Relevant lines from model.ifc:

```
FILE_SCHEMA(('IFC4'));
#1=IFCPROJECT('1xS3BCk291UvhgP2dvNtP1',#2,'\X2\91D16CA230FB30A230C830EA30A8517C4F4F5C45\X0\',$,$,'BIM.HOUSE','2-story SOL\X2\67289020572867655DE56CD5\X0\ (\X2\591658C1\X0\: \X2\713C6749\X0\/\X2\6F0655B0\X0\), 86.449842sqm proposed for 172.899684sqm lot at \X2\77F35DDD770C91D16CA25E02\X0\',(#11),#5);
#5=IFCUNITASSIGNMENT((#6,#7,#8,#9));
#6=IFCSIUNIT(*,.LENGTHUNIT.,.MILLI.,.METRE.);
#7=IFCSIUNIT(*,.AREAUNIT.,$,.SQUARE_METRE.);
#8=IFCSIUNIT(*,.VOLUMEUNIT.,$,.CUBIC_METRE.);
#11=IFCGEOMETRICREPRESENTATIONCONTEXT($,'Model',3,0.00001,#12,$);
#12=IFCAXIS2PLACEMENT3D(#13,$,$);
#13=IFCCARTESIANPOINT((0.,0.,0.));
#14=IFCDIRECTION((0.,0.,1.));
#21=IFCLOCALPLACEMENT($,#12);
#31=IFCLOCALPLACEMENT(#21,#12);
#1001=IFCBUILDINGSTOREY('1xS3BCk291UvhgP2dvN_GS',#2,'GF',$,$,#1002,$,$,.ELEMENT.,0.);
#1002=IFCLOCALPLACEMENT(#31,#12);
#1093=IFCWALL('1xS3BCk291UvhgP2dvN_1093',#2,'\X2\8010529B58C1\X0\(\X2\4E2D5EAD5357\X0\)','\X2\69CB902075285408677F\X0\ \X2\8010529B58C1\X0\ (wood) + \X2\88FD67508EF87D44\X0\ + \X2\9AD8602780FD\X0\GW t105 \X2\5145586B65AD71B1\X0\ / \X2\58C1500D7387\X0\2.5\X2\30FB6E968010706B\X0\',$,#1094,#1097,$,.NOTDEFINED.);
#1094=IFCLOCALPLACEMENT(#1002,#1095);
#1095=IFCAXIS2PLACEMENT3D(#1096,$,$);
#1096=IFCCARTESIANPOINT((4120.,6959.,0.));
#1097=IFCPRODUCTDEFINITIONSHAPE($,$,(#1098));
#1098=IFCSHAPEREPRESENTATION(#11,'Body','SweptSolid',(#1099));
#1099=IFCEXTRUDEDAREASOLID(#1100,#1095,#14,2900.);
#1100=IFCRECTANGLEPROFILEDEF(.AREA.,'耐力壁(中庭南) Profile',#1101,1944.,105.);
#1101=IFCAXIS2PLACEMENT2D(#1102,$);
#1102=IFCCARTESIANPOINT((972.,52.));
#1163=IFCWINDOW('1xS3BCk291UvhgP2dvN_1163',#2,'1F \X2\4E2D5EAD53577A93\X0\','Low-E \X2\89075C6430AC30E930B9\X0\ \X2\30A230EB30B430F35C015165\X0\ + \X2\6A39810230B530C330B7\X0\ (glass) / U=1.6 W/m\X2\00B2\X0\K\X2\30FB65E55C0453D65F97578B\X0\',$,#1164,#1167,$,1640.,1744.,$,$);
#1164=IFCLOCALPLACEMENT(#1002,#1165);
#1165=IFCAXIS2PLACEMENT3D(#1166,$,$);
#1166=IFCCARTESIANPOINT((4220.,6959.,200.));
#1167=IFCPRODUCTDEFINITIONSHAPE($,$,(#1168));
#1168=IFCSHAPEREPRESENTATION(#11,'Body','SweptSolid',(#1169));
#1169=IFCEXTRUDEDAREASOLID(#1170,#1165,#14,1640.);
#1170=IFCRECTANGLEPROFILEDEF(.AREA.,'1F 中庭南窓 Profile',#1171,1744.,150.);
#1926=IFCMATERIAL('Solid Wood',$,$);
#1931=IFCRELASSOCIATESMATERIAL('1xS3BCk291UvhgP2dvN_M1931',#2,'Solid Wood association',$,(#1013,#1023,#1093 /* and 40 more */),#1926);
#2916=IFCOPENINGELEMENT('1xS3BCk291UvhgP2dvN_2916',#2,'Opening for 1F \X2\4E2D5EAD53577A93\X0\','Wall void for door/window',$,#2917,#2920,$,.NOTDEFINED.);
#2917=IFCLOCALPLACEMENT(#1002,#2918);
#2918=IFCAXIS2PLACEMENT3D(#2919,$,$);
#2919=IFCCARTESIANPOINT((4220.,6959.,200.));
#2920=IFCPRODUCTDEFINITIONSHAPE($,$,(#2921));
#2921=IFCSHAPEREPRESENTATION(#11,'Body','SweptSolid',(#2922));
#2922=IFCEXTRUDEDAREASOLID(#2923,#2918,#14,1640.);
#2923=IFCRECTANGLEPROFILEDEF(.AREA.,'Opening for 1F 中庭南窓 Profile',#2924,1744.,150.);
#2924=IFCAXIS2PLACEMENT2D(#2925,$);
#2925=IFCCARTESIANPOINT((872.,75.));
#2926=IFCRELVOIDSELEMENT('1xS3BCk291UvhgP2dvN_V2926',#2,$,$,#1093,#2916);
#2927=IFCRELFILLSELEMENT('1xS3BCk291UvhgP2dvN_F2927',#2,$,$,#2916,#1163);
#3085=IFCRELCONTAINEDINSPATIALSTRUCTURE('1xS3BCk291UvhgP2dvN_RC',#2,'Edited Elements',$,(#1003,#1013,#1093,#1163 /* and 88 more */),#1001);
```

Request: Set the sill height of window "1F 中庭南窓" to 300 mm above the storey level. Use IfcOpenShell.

```python
import numpy as np
import ifcopenshell
import ifcopenshell.api.geometry
import ifcopenshell.geom
import ifcopenshell.util.element
import ifcopenshell.util.placement
import ifcopenshell.util.shape
import ifcopenshell.util.unit

model = ifcopenshell.open("model.ifc")
unit_scale = ifcopenshell.util.unit.calculate_unit_scale(model)

window = model.by_guid("1xS3BCk291UvhgP2dvN_1163")
opening = window.FillsVoids[0].RelatingOpeningElement
storey = ifcopenshell.util.element.get_container(window, ifc_class="IfcBuildingStorey")
level = ifcopenshell.util.placement.get_local_placement(storey.ObjectPlacement)[2, 3]

# The opening's origin need not be at the sill, so measure its lowest point.
shape = ifcopenshell.geom.create_shape(ifcopenshell.geom.settings(), opening)
bottom = ifcopenshell.util.shape.get_shape_bottom_elevation(shape, shape.geometry) / unit_scale
dz = level + 300.0 - bottom

shift = np.array([0.0, 0.0, dz])
# The window is not placed relative to its opening, so move both.
for product in (opening, window):
    matrix = ifcopenshell.util.placement.get_local_placement(product.ObjectPlacement)
    matrix[:3, 3] += shift
    ifcopenshell.api.geometry.edit_object_placement(model, product=product, matrix=matrix, is_si=False)

print(f"moved by {dz * unit_scale:+.3f} m")

model.write("model_rev.ifc")
```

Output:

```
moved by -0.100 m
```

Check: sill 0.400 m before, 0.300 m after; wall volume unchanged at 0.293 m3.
